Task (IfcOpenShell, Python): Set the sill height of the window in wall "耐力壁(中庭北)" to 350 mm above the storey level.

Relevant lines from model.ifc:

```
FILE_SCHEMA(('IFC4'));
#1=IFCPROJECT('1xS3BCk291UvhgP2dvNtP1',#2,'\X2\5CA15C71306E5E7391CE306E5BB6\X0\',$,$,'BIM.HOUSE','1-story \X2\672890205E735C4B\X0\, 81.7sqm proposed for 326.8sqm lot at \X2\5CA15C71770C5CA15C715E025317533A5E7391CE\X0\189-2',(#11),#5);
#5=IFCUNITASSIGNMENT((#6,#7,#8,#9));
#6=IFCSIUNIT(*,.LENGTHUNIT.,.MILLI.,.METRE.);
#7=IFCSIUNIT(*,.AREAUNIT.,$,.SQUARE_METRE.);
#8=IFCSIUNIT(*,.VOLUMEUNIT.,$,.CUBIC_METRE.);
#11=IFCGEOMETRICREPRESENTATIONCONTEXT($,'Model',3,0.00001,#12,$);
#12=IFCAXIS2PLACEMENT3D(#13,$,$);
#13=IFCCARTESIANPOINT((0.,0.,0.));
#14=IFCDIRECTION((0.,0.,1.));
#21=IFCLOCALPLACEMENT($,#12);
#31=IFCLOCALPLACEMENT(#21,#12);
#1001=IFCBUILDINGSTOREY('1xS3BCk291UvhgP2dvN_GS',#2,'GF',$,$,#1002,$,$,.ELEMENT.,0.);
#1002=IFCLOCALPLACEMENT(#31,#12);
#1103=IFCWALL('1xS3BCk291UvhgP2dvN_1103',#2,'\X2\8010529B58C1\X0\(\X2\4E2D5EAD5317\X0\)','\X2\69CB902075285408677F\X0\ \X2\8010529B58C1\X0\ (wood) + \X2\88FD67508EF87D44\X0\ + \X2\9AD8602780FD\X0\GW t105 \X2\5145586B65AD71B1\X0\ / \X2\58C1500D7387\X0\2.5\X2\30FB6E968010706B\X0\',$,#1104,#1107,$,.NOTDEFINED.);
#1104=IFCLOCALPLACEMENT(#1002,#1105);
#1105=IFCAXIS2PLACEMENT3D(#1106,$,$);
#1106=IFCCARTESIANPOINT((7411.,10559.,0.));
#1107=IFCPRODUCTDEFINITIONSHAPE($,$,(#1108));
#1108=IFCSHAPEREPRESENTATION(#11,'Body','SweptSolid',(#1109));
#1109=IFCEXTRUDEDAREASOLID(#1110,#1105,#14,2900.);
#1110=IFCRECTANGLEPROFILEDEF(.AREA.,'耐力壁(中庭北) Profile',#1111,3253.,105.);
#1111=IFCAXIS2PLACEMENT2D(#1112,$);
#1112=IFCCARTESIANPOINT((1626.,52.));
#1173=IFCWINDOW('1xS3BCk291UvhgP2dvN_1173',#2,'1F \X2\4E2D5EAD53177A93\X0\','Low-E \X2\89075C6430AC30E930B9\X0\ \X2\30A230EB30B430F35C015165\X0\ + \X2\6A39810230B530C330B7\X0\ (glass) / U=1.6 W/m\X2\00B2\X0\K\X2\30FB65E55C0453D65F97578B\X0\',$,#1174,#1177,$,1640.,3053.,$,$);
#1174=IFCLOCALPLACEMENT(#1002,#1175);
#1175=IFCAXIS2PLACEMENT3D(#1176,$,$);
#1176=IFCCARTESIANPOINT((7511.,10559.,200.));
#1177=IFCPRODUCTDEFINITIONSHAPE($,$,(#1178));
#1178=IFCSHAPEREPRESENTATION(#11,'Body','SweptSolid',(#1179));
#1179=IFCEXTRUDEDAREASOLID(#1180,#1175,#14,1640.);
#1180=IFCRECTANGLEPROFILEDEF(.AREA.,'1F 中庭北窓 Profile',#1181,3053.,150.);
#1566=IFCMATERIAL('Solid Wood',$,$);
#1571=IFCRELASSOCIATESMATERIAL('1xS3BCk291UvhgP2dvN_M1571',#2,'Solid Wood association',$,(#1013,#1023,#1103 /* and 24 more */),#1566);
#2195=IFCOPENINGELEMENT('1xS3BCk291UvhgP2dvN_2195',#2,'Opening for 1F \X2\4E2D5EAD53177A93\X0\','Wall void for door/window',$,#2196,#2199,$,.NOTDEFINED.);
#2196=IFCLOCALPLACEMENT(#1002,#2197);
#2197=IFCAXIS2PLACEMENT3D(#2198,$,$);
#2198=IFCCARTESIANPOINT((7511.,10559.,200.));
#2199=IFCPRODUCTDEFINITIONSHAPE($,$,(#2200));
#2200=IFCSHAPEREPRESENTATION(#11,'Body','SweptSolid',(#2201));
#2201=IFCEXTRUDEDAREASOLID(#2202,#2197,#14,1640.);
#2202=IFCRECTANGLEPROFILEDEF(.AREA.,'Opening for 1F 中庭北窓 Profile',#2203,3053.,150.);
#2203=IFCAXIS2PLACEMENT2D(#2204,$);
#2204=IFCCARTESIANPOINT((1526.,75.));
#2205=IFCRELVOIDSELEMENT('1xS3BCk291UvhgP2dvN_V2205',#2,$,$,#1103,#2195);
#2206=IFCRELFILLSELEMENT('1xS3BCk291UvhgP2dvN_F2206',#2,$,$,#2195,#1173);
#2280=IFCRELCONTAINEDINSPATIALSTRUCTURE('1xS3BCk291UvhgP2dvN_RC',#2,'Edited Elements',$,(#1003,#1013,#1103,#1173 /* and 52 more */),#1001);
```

```python
import numpy as np
import ifcopenshell
import ifcopenshell.api.geometry
import ifcopenshell.geom
import ifcopenshell.util.element
import ifcopenshell.util.placement
import ifcopenshell.util.shape
import ifcopenshell.util.unit

model = ifcopenshell.open("model.ifc")
unit_scale = ifcopenshell.util.unit.calculate_unit_scale(model)

window = model.by_guid("1xS3BCk291UvhgP2dvN_1173")
opening = window.FillsVoids[0].RelatingOpeningElement
storey = ifcopenshell.util.element.get_container(window, ifc_class="IfcBuildingStorey")
level = ifcopenshell.util.placement.get_local_placement(storey.ObjectPlacement)[2, 3]

# The opening's origin need not be at the sill, so measure its lowest point.
shape = ifcopenshell.geom.create_shape(ifcopenshell.geom.settings(), opening)
bottom = ifcopenshell.util.shape.get_shape_bottom_elevation(shape, shape.geometry) / unit_scale
dz = level + 0.35 / unit_scale - bottom

shift = np.array([0.0, 0.0, dz])
# The window is not placed relative to its opening, so move both.
for product in (opening, window):
    matrix = ifcopenshell.util.placement.get_local_placement(product.ObjectPlacement)
    matrix[:3, 3] += shift
    ifcopenshell.api.geometry.edit_object_placement(model, product=product, matrix=matrix, is_si=False)

print(f"moved by {dz * unit_scale:+.3f} m")

model.write("model_edited.ifc")
```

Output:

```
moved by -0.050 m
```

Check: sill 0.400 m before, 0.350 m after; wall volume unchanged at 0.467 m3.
